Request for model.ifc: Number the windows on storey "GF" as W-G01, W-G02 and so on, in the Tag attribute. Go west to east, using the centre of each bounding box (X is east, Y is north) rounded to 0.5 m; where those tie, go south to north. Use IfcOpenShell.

First a look at what the model holds.

```python
import ifcopenshell
import ifcopenshell.util.element
import ifcopenshell.util.placement

model = ifcopenshell.open("model.ifc")
print(model.schema)
storey = next(s for s in model.by_type("IfcBuildingStorey") if s.Name == "GF")
windows = [e for e in ifcopenshell.util.element.get_decomposition(storey) if e.is_a("IfcWindow")]
for e in sorted(windows, key=lambda e: e.id()):
    origin = ifcopenshell.util.placement.get_local_placement(e.ObjectPlacement)[:3, 3]
    print(e.id(), e.Tag, e.Name, origin.round(2) + 0.0, sep=" | ")
```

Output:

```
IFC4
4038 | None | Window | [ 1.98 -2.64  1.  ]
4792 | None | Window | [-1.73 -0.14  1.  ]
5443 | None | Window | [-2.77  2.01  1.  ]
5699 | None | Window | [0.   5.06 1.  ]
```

```python
import ifcopenshell
import ifcopenshell.geom
import ifcopenshell.util.element
import ifcopenshell.util.shape

model = ifcopenshell.open("model.ifc")
settings = ifcopenshell.geom.settings()
settings.set("use-world-coords", True)


def centre(element):
    shape = ifcopenshell.geom.create_shape(settings, element)
    return ifcopenshell.util.shape.get_bbox_centroid(shape.geometry)


storey = next(s for s in model.by_type("IfcBuildingStorey") if s.Name == "GF")
windows = [e for e in ifcopenshell.util.element.get_decomposition(storey) if e.is_a("IfcWindow")]

# Insertion points can sit at a corner or the storey origin, so sort by the geometry (in metres).
centres = {e: centre(e) for e in windows}
windows.sort(key=lambda e: (round(centres[e][0] / 0.5), centres[e][1]))

for i, e in enumerate(windows, start=1):
    number = f"W-G{i:02d}"
    e.Tag = number
    print(e.id(), number)

model.write("model_edited.ifc")
```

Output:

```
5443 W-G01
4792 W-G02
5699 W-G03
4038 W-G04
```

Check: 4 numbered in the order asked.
